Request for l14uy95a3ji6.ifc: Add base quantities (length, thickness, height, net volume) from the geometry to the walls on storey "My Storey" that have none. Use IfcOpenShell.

First a look at what the model holds.

```python
import ifcopenshell
import ifcopenshell.util.element
import ifcopenshell.util.unit

model = ifcopenshell.open("l14uy95a3ji6.ifc")
print(model.schema)
for unit_type in ("LENGTHUNIT", "AREAUNIT", "VOLUMEUNIT"):
    print(unit_type, ifcopenshell.util.unit.calculate_unit_scale(model, unit_type))
storey = next(s for s in model.by_type("IfcBuildingStorey") if s.Name == "My Storey")
walls = [e for e in ifcopenshell.util.element.get_decomposition(storey) if e.is_a("IfcWall")]
for e in sorted(walls, key=lambda e: e.id()):
    print(e.id(), e.is_a(), e.Name, list(ifcopenshell.util.element.get_psets(e, qtos_only=True)), sep=" | ")
```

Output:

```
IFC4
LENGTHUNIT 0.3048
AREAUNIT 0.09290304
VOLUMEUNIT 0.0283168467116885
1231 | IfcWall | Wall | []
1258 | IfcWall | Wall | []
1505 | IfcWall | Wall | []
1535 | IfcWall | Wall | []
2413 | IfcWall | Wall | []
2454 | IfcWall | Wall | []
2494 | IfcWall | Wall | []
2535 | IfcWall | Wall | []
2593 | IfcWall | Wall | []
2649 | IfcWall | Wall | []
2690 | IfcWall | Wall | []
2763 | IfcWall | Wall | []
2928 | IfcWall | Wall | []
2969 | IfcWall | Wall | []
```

```python
import ifcopenshell
import ifcopenshell.api.pset
import ifcopenshell.geom
import ifcopenshell.util.element
import ifcopenshell.util.shape
import ifcopenshell.util.unit

model = ifcopenshell.open("l14uy95a3ji6.ifc")
unit_scale = ifcopenshell.util.unit.calculate_unit_scale(model)
volume_scale = ifcopenshell.util.unit.calculate_unit_scale(model, "VOLUMEUNIT")
settings = ifcopenshell.geom.settings()

storey = next(s for s in model.by_type("IfcBuildingStorey") if s.Name == "My Storey")
walls = [e for e in ifcopenshell.util.element.get_decomposition(storey) if e.is_a("IfcWall")]

for e in sorted(walls, key=lambda e: e.id()):
    if ifcopenshell.util.element.get_psets(e, qtos_only=True, should_inherit=False):
        continue
    # Geometry comes back in metres, in the element's own axes.
    shape = ifcopenshell.geom.create_shape(settings, e)
    values = {
        "Length": ifcopenshell.util.shape.get_x(shape.geometry) / unit_scale,
        "Width": ifcopenshell.util.shape.get_y(shape.geometry) / unit_scale,
        "Height": ifcopenshell.util.shape.get_z(shape.geometry) / unit_scale,
        "NetVolume": ifcopenshell.util.shape.get_volume(shape.geometry) / volume_scale,
    }
    qto = ifcopenshell.api.pset.add_qto(model, product=e, name="Qto_WallBaseQuantities")
    ifcopenshell.api.pset.edit_qto(model, qto=qto, properties=values)
    print(e.id(), {k: round(v, 3) for k, v in values.items()})

model.write("l14uy95a3ji6-out.ifc")
```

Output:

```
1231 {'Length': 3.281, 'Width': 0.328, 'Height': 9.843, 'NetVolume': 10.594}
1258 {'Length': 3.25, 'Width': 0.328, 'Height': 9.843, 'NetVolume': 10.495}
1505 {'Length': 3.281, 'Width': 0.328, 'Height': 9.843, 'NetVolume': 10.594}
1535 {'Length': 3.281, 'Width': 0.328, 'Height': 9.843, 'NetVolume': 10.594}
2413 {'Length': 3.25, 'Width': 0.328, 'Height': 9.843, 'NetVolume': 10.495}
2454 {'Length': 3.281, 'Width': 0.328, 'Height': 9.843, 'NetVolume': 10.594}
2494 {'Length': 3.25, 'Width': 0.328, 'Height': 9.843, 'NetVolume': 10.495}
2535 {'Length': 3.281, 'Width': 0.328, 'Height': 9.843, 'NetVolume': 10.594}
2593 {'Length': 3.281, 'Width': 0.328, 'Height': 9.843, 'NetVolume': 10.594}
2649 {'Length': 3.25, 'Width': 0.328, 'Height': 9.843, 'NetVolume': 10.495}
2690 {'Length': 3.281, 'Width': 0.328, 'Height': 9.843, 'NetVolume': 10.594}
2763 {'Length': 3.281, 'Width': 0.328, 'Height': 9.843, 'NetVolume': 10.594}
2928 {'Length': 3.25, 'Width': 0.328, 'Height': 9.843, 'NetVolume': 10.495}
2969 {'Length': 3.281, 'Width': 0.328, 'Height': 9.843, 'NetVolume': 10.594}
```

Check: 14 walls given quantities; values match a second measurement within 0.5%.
